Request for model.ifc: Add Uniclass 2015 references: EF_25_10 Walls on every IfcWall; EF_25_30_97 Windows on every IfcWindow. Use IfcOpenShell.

First a look at what the model holds.

```python
import ifcopenshell

model = ifcopenshell.open("model.ifc")
print(model.schema)
print("classifications:", [c.Name for c in model.by_type("IfcClassification")])
for ifc_class in ("IfcDoor", "IfcRoof", "IfcStair", "IfcWall", "IfcWindow"):
    print(ifc_class, len(model.by_type(ifc_class)))
```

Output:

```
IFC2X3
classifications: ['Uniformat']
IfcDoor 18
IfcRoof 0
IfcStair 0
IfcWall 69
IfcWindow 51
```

```python
import ifcopenshell
import ifcopenshell.api.classification

model = ifcopenshell.open("model.ifc")

# IFC2X3 requires Source and Edition and has no link from the project to the system.
system = model.create_entity("IfcClassification", Source="NBS", Edition="2015", Name="Uniclass 2015")

codes = {
    "IfcWall": ("EF_25_10", "Walls"),
    "IfcWindow": ("EF_25_30_97", "Windows"),
}
for ifc_class, (code, name) in codes.items():
    products = model.by_type(ifc_class)
    ifcopenshell.api.classification.add_reference(
        model, products=products, classification=system, identification=code, name=name
    )
    print(code, len(products))

model.write("model_rev.ifc")
```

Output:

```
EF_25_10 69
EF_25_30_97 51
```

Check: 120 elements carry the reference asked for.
